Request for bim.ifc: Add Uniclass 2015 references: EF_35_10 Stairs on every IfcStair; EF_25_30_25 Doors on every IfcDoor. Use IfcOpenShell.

First a look at what the model holds.

```python
import ifcopenshell

model = ifcopenshell.open("bim.ifc")
print(model.schema)
print("classifications:", [c.Name for c in model.by_type("IfcClassification")])
for ifc_class in ("IfcDoor", "IfcRoof", "IfcStair", "IfcWall", "IfcWindow"):
    print(ifc_class, len(model.by_type(ifc_class)))
```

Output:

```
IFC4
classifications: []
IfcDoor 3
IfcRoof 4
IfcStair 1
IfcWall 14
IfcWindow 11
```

```python
import ifcopenshell
import ifcopenshell.api.classification

model = ifcopenshell.open("bim.ifc")

system = ifcopenshell.api.classification.add_classification(model, classification="Uniclass 2015")

codes = {
    "IfcStair": ("EF_35_10", "Stairs"),
    "IfcDoor": ("EF_25_30_25", "Doors"),
}
for ifc_class, (code, name) in codes.items():
    products = model.by_type(ifc_class)
    ifcopenshell.api.classification.add_reference(
        model, products=products, classification=system, identification=code, name=name
    )
    print(code, len(products))

model.write("bim_updated.ifc")
```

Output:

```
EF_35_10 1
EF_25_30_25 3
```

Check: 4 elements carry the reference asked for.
